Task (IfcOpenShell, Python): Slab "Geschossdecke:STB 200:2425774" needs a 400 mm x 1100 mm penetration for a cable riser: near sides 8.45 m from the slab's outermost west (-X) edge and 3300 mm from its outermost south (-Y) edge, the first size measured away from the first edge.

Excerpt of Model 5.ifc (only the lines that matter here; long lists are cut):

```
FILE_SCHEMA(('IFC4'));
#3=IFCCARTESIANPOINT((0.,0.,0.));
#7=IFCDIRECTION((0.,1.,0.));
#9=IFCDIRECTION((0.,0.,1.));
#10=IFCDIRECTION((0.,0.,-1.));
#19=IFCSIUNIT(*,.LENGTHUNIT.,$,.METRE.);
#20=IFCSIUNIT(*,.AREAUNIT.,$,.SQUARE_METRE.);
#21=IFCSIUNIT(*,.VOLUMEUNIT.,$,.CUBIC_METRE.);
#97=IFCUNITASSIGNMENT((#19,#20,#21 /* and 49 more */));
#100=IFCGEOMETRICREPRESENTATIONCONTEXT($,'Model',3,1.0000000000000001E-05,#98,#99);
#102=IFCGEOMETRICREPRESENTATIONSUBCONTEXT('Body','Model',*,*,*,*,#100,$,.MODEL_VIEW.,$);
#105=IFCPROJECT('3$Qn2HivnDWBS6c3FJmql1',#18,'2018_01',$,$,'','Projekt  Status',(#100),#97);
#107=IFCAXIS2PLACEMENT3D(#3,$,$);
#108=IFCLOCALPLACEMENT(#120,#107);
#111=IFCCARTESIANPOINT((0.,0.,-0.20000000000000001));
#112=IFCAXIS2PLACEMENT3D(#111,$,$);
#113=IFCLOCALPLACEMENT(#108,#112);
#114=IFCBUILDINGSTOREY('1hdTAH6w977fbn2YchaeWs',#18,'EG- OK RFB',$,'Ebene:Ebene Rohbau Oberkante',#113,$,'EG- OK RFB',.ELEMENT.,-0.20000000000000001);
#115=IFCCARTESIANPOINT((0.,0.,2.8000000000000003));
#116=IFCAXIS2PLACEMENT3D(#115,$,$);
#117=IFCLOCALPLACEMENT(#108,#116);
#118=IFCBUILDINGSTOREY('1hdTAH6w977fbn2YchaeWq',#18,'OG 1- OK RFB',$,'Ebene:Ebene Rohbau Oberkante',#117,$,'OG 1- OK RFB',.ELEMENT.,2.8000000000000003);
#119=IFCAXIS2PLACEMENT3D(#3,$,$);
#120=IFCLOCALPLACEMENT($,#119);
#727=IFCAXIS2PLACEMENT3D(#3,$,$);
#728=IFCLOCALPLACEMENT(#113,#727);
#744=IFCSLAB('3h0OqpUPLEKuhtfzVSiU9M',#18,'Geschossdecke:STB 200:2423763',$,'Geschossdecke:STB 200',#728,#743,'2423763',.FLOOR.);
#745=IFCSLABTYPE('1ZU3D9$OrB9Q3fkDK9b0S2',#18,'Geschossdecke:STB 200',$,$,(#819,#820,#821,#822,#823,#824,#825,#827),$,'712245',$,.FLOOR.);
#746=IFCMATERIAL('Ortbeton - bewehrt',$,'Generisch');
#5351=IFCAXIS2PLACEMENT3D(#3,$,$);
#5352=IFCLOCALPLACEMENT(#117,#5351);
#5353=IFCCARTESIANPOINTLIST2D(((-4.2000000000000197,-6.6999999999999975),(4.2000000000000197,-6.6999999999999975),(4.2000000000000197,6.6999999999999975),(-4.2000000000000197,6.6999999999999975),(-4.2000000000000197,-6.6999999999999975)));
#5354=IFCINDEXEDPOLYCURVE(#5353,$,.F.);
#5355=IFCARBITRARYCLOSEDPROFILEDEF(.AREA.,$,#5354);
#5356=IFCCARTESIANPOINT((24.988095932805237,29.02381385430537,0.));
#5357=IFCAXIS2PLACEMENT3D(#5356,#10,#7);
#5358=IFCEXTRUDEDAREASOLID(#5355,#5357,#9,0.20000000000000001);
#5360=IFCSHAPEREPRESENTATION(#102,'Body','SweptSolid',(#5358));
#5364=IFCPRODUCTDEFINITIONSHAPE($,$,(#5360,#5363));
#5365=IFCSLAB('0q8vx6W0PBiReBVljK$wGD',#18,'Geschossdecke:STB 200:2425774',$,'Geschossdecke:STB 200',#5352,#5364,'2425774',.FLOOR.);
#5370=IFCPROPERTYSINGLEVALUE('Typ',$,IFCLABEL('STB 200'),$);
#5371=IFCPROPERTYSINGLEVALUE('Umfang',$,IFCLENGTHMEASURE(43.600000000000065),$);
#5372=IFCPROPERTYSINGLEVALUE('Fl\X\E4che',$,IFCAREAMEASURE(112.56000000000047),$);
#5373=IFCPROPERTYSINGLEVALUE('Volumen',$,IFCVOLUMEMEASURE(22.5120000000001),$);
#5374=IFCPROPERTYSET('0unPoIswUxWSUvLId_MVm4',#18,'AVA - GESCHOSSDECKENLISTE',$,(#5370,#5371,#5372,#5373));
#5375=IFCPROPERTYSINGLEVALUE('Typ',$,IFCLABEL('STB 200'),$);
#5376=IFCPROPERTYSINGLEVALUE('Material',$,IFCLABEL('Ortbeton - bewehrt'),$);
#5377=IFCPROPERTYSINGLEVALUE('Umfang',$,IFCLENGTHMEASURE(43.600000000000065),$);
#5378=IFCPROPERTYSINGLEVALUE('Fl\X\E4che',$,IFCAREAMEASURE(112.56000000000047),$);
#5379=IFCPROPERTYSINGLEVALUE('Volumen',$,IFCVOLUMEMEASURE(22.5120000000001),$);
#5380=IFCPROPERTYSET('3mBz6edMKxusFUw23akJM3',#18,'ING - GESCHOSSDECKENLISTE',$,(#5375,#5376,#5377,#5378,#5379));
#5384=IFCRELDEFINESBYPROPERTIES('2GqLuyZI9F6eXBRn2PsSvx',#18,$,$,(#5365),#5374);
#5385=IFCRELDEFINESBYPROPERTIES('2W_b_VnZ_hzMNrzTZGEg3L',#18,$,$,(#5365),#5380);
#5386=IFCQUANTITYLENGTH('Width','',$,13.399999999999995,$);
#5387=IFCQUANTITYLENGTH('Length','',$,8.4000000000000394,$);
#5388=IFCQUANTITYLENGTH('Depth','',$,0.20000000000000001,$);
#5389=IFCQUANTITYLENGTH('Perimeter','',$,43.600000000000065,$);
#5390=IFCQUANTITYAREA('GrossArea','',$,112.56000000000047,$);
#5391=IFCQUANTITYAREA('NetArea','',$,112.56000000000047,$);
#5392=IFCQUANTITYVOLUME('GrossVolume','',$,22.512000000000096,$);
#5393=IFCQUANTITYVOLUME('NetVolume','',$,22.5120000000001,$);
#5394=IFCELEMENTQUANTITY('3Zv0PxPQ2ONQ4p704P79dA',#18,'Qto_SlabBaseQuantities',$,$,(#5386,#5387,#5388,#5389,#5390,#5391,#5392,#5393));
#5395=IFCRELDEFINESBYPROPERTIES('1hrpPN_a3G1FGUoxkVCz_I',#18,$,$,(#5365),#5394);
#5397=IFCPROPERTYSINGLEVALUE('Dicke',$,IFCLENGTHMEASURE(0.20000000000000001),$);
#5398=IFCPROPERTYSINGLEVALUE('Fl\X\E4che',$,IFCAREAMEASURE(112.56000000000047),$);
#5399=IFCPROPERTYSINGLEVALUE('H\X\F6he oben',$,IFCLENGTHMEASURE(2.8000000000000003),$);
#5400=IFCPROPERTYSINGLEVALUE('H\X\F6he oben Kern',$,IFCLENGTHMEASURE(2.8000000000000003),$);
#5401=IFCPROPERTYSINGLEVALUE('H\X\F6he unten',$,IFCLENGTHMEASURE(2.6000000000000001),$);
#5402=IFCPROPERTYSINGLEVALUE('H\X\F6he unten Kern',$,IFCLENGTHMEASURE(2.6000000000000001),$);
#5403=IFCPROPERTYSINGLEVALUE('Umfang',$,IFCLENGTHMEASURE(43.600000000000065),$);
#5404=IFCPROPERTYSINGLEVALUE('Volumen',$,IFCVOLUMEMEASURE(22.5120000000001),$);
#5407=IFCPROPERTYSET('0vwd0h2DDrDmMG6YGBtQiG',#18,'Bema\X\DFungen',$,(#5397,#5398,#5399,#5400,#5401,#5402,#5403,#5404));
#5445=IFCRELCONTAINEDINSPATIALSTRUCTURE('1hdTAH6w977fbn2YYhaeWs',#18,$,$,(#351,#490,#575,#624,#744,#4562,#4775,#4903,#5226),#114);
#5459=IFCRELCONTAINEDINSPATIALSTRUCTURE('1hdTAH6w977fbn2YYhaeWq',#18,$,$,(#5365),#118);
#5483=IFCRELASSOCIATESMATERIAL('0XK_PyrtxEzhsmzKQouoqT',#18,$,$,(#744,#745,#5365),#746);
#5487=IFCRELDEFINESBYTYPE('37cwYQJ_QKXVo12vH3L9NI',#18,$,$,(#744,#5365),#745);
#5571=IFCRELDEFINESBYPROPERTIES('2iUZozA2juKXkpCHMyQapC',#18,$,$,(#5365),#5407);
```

```python
import numpy as np
import ifcopenshell
import ifcopenshell.api.feature
import ifcopenshell.api.geometry
import ifcopenshell.api.pset
import ifcopenshell.api.root
import ifcopenshell.geom
import ifcopenshell.util.element
import ifcopenshell.util.placement
import ifcopenshell.util.representation
import ifcopenshell.util.shape
import ifcopenshell.util.unit

model = ifcopenshell.open("Model 5.ifc")
unit_scale = ifcopenshell.util.unit.calculate_unit_scale(model)
area_scale = ifcopenshell.util.unit.calculate_unit_scale(model, "AREAUNIT")
volume_scale = ifcopenshell.util.unit.calculate_unit_scale(model, "VOLUMEUNIT")
settings = ifcopenshell.geom.settings()


def volume(element):
    """Net volume in cubic metres, openings subtracted."""
    shape = ifcopenshell.geom.create_shape(settings, element)
    return ifcopenshell.util.shape.get_volume(shape.geometry)


slab = model.by_guid("0q8vx6W0PBiReBVljK$wGD")
before = volume(slab)

# Extent in the slab's own axes, in metres. The edges named are its -X and -Y sides.
slab_shape = ifcopenshell.geom.create_shape(settings, slab)
vertices = ifcopenshell.util.shape.get_vertices(slab_shape.geometry)
x_min, y_min, bottom = vertices.min(axis=0)
top = vertices[:, 2].max()

opening = ifcopenshell.api.root.create_entity(model, ifc_class="IfcOpeningElement", name="Cable riser opening", predefined_type="OPENING")
context = ifcopenshell.util.representation.get_context(model, "Model", "Body", "MODEL_VIEW")
width, depth = 0.4, 1.1
outline = [(0.0, 0.0), (width, 0.0), (width, depth), (0.0, depth), (0.0, 0.0)]
# Overshoot both faces by 50 mm so the cut is clean.
shape = ifcopenshell.api.geometry.add_slab_representation(
    model, context=context, depth=top - bottom + 0.1, polyline=outline
)
ifcopenshell.api.geometry.assign_representation(model, product=opening, representation=shape)

matrix = ifcopenshell.util.placement.get_local_placement(slab.ObjectPlacement)
matrix[:, 3] = matrix @ np.append(np.array([x_min + 8.45, y_min + 3.3, bottom - 0.05]) / unit_scale, 1.0)
ifcopenshell.api.geometry.edit_object_placement(model, product=opening, matrix=matrix, is_si=False)
ifcopenshell.api.feature.add_feature(model, feature=opening, element=slab)

after = volume(slab)

# Update the slab's stored quantities.
pset = model.by_id(ifcopenshell.util.element.get_pset(slab, "AVA - GESCHOSSDECKENLISTE", should_inherit=False)["id"])
ifcopenshell.api.pset.edit_pset(model, pset=pset, properties={
    "Fläche": model.create_entity("IfcAreaMeasure", after / (top - bottom) / area_scale),
    "Volumen": model.create_entity("IfcVolumeMeasure", after / volume_scale),
})
pset = model.by_id(ifcopenshell.util.element.get_pset(slab, "ING - GESCHOSSDECKENLISTE", should_inherit=False)["id"])
ifcopenshell.api.pset.edit_pset(model, pset=pset, properties={
    "Fläche": model.create_entity("IfcAreaMeasure", after / (top - bottom) / area_scale),
    "Volumen": model.create_entity("IfcVolumeMeasure", after / volume_scale),
})
qto = model.by_id(ifcopenshell.util.element.get_pset(slab, "Qto_SlabBaseQuantities", should_inherit=False)["id"])
ifcopenshell.api.pset.edit_qto(model, qto=qto, properties={
    "NetArea": after / (top - bottom) / area_scale,
    "NetVolume": after / volume_scale,
})
pset = model.by_id(ifcopenshell.util.element.get_pset(slab, "Bemaßungen", should_inherit=False)["id"])
ifcopenshell.api.pset.edit_pset(model, pset=pset, properties={
    "Fläche": model.create_entity("IfcAreaMeasure", after / (top - bottom) / area_scale),
    "Volumen": model.create_entity("IfcVolumeMeasure", after / volume_scale),
})

print(f"slab volume {before:.3f} -> {after:.3f} m3")

model.write("Model 5_v2.ifc")
```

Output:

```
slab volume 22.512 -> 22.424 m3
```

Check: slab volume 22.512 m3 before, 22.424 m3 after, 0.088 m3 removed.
